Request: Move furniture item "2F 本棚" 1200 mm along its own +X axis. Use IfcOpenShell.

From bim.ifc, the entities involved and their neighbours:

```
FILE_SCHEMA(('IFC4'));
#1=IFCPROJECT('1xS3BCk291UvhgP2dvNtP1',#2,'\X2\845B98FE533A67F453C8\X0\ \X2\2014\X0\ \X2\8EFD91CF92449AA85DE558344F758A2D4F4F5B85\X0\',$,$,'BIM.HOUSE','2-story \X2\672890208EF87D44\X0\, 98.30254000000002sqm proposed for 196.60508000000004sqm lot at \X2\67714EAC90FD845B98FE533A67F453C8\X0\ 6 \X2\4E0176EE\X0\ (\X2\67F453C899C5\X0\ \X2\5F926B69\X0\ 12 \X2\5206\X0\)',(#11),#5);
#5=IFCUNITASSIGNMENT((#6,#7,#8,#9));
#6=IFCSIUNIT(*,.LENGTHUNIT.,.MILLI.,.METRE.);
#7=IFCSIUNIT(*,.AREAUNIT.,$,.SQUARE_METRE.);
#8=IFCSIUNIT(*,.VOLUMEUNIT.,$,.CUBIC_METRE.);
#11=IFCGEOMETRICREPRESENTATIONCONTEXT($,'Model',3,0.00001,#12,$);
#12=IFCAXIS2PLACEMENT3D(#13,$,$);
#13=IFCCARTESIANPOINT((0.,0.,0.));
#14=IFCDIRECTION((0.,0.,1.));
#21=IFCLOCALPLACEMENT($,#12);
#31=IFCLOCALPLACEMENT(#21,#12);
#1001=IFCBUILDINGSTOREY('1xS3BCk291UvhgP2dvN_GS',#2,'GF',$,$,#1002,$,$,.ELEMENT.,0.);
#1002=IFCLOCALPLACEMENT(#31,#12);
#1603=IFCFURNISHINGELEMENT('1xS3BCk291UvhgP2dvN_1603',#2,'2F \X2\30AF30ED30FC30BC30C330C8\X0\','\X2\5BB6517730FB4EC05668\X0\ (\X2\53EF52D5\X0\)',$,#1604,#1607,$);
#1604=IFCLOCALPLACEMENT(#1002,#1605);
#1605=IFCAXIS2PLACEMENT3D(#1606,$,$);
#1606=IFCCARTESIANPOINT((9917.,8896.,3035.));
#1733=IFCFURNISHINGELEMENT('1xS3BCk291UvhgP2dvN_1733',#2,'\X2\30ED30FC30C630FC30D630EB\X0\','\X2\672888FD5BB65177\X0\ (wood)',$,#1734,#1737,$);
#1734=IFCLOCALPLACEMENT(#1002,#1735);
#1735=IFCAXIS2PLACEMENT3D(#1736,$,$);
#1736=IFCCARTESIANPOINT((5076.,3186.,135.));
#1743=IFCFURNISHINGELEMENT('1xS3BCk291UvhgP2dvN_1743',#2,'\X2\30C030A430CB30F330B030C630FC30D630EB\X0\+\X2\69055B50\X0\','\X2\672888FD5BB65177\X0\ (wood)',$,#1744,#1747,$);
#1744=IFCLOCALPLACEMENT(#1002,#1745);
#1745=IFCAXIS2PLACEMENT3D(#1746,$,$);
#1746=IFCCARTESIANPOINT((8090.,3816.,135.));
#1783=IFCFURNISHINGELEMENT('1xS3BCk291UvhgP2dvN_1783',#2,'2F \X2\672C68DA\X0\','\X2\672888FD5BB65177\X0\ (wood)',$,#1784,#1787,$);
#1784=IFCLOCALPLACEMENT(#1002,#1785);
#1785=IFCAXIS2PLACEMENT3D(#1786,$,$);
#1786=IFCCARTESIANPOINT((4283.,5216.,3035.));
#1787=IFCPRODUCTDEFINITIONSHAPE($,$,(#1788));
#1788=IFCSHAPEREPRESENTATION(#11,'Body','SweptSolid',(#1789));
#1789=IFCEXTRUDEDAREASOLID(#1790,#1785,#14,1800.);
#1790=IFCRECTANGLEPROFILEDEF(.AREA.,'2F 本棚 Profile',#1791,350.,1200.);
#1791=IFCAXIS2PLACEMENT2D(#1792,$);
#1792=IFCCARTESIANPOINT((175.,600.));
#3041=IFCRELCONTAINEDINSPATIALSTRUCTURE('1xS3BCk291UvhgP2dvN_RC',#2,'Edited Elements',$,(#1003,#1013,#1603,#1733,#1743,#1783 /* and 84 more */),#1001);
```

```python
import ifcopenshell
import ifcopenshell.api.geometry
import ifcopenshell.util.placement

model = ifcopenshell.open("bim.ifc")

item = model.by_guid("1xS3BCk291UvhgP2dvN_1783")
matrix = ifcopenshell.util.placement.get_local_placement(item.ObjectPlacement)
matrix[:3, 3] += matrix[:3, 0] * 1200.0
ifcopenshell.api.geometry.edit_object_placement(model, product=item, matrix=matrix, is_si=False)

print(ifcopenshell.util.placement.get_local_placement(item.ObjectPlacement).round(3) + 0.0)

model.write("bim_rev.ifc")
```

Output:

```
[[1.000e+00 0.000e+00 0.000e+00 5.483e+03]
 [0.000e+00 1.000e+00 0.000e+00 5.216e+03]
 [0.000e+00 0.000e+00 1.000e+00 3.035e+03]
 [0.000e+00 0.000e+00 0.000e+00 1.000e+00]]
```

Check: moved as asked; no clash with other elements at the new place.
